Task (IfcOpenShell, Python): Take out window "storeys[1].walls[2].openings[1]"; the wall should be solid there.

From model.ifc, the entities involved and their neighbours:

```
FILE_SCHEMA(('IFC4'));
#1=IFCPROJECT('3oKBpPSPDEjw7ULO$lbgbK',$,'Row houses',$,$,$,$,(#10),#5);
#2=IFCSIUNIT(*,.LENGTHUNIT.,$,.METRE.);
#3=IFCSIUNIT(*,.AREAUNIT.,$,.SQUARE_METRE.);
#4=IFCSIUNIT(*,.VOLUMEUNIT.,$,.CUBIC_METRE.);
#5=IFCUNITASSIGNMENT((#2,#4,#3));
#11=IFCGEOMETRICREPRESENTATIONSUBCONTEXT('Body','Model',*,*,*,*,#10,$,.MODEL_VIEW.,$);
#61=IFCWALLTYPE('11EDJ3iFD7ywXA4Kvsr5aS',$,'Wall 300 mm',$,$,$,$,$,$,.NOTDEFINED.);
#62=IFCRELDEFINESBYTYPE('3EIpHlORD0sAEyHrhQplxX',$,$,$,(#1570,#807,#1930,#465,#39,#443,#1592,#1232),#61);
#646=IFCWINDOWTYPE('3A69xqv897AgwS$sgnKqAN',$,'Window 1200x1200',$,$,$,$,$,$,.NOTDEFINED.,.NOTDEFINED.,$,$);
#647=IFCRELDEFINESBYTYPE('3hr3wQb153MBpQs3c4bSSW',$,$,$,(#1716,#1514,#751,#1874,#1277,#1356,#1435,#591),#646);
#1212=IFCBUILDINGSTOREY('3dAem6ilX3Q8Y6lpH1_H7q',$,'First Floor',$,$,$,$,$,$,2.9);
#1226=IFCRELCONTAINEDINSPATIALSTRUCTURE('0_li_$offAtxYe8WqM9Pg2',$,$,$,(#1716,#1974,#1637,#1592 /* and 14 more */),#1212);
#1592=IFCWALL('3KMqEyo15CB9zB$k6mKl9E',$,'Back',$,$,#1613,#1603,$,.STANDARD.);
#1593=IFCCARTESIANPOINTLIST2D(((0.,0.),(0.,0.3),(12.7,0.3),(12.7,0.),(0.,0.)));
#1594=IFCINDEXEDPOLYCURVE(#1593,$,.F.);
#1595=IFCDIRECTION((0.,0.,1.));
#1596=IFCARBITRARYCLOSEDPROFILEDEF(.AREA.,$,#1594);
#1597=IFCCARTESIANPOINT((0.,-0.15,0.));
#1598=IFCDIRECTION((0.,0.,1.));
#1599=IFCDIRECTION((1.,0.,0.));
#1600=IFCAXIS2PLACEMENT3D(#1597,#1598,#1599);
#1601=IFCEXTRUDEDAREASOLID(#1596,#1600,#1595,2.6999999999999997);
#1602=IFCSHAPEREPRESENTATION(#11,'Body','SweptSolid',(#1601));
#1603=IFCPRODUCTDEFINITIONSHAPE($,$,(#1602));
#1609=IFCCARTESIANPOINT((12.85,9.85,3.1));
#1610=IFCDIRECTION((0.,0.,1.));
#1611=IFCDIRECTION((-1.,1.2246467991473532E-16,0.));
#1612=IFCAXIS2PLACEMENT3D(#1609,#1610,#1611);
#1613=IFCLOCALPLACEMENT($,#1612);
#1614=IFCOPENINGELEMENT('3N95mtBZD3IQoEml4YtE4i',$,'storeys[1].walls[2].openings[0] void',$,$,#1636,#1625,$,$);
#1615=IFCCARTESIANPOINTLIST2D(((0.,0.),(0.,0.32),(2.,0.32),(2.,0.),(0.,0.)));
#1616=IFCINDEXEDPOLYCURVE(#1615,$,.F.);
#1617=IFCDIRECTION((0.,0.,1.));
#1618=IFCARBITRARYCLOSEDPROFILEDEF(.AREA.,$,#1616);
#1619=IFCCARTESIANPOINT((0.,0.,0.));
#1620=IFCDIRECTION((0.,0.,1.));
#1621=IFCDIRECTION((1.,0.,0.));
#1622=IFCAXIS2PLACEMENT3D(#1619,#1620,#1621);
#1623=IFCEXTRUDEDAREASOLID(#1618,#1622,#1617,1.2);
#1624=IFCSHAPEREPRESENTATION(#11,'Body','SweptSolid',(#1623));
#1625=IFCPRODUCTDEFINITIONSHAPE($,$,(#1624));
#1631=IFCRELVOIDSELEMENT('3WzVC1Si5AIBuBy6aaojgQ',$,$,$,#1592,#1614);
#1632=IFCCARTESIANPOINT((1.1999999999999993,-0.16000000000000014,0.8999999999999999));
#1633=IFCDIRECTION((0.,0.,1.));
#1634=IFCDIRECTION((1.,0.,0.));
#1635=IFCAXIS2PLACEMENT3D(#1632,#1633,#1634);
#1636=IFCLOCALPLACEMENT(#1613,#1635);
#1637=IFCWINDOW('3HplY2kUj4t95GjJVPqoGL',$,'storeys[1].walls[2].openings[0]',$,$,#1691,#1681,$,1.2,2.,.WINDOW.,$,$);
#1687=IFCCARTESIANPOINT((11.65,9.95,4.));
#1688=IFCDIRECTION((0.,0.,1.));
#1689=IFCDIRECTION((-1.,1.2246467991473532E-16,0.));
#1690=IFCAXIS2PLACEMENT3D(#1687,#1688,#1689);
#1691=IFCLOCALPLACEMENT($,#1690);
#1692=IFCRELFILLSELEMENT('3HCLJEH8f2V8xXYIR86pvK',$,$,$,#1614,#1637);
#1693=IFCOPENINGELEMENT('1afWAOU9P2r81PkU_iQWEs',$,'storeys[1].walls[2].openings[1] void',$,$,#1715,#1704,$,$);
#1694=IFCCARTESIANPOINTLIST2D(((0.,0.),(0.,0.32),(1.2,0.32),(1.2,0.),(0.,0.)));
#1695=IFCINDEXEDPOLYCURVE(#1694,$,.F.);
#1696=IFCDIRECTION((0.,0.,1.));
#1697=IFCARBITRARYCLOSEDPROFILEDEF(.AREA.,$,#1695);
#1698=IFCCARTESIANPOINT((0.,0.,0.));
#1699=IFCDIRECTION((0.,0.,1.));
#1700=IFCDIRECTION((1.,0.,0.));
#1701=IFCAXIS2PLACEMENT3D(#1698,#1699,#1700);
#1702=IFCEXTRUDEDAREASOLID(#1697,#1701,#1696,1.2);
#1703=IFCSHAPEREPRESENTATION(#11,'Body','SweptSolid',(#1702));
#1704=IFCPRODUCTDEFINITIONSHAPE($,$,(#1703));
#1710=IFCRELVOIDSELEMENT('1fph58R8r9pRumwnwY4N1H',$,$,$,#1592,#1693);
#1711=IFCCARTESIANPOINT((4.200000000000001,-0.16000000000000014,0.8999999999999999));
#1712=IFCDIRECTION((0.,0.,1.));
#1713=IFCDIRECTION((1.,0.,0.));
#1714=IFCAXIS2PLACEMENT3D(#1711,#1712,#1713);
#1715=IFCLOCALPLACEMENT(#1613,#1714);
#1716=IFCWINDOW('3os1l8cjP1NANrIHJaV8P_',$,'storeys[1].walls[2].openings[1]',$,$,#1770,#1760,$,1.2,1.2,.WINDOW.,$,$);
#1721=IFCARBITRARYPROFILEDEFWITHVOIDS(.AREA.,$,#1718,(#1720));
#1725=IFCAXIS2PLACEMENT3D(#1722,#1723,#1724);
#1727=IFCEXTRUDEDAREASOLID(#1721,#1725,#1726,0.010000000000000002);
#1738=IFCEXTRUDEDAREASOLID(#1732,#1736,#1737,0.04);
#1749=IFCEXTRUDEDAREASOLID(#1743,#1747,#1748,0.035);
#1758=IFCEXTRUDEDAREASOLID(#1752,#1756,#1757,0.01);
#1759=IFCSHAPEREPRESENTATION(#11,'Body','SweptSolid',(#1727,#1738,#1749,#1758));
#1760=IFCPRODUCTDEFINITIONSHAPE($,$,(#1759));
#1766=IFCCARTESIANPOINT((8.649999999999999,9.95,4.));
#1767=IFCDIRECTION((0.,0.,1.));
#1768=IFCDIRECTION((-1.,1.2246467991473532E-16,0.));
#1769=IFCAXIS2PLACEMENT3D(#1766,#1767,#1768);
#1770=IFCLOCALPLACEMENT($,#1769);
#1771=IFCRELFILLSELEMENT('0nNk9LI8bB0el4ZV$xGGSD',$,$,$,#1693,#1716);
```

```python
import ifcopenshell
import ifcopenshell.api.feature
import ifcopenshell.api.root
import ifcopenshell.geom
import ifcopenshell.util.shape

model = ifcopenshell.open("model.ifc")
settings = ifcopenshell.geom.settings()


def volume(element):
    """Net volume in cubic metres, openings subtracted."""
    shape = ifcopenshell.geom.create_shape(settings, element)
    return ifcopenshell.util.shape.get_volume(shape.geometry)


window = model.by_id(1716)
opening = window.FillsVoids[0].RelatingOpeningElement
wall = opening.VoidsElements[0].RelatingBuildingElement
before = volume(wall)

ifcopenshell.api.root.remove_product(model, product=window)
ifcopenshell.api.feature.remove_feature(model, feature=opening)

after = volume(wall)

print(f"wall volume {before:.3f} -> {after:.3f} m3")

model.write("model-out.ifc")
```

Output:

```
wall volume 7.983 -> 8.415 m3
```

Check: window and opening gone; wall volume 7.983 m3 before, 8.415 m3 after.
